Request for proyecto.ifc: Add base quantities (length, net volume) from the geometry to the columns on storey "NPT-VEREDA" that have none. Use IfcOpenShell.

First a look at what the model holds.

```python
import ifcopenshell
import ifcopenshell.util.element
import ifcopenshell.util.unit

model = ifcopenshell.open("proyecto.ifc")
print(model.schema)
for unit_type in ("LENGTHUNIT", "AREAUNIT", "VOLUMEUNIT"):
    print(unit_type, ifcopenshell.util.unit.calculate_unit_scale(model, unit_type))
storey = next(s for s in model.by_type("IfcBuildingStorey") if s.Name == "NPT-VEREDA")
columns = [e for e in ifcopenshell.util.element.get_decomposition(storey) if e.is_a("IfcColumn")]
for e in sorted(columns, key=lambda e: e.id()):
    print(e.id(), e.is_a(), e.Name, list(ifcopenshell.util.element.get_psets(e, qtos_only=True)), sep=" | ")
```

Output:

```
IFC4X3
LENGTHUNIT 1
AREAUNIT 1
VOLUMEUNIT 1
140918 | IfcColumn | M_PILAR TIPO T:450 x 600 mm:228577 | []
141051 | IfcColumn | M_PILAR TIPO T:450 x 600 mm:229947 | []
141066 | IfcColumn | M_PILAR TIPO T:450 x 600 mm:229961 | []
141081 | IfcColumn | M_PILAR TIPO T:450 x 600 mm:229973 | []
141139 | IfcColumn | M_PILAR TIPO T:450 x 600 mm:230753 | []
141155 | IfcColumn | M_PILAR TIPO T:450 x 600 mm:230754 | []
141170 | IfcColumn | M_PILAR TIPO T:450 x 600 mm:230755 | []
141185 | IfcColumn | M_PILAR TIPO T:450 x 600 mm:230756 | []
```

```python
import ifcopenshell
import ifcopenshell.api.pset
import ifcopenshell.geom
import ifcopenshell.util.element
import ifcopenshell.util.shape
import ifcopenshell.util.unit

model = ifcopenshell.open("proyecto.ifc")
unit_scale = ifcopenshell.util.unit.calculate_unit_scale(model)
volume_scale = ifcopenshell.util.unit.calculate_unit_scale(model, "VOLUMEUNIT")
settings = ifcopenshell.geom.settings()

storey = next(s for s in model.by_type("IfcBuildingStorey") if s.Name == "NPT-VEREDA")
columns = [e for e in ifcopenshell.util.element.get_decomposition(storey) if e.is_a("IfcColumn")]

for e in sorted(columns, key=lambda e: e.id()):
    if ifcopenshell.util.element.get_psets(e, qtos_only=True, should_inherit=False):
        continue
    # Geometry comes back in metres, in the element's own axes.
    shape = ifcopenshell.geom.create_shape(settings, e)
    values = {
        "Length": ifcopenshell.util.shape.get_z(shape.geometry) / unit_scale,
        "NetVolume": ifcopenshell.util.shape.get_volume(shape.geometry) / volume_scale,
    }
    qto = ifcopenshell.api.pset.add_qto(model, product=e, name="Qto_ColumnBaseQuantities")
    ifcopenshell.api.pset.edit_qto(model, qto=qto, properties=values)
    print(e.id(), {k: round(v, 3) for k, v in values.items()})

model.write("proyecto_edited.ifc")
```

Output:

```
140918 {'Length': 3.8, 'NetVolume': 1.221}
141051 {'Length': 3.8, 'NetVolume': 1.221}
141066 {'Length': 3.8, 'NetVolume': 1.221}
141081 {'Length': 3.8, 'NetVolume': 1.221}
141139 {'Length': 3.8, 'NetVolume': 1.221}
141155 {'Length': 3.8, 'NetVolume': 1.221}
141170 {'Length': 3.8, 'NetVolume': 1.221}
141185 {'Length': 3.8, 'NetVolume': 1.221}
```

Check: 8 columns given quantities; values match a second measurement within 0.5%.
